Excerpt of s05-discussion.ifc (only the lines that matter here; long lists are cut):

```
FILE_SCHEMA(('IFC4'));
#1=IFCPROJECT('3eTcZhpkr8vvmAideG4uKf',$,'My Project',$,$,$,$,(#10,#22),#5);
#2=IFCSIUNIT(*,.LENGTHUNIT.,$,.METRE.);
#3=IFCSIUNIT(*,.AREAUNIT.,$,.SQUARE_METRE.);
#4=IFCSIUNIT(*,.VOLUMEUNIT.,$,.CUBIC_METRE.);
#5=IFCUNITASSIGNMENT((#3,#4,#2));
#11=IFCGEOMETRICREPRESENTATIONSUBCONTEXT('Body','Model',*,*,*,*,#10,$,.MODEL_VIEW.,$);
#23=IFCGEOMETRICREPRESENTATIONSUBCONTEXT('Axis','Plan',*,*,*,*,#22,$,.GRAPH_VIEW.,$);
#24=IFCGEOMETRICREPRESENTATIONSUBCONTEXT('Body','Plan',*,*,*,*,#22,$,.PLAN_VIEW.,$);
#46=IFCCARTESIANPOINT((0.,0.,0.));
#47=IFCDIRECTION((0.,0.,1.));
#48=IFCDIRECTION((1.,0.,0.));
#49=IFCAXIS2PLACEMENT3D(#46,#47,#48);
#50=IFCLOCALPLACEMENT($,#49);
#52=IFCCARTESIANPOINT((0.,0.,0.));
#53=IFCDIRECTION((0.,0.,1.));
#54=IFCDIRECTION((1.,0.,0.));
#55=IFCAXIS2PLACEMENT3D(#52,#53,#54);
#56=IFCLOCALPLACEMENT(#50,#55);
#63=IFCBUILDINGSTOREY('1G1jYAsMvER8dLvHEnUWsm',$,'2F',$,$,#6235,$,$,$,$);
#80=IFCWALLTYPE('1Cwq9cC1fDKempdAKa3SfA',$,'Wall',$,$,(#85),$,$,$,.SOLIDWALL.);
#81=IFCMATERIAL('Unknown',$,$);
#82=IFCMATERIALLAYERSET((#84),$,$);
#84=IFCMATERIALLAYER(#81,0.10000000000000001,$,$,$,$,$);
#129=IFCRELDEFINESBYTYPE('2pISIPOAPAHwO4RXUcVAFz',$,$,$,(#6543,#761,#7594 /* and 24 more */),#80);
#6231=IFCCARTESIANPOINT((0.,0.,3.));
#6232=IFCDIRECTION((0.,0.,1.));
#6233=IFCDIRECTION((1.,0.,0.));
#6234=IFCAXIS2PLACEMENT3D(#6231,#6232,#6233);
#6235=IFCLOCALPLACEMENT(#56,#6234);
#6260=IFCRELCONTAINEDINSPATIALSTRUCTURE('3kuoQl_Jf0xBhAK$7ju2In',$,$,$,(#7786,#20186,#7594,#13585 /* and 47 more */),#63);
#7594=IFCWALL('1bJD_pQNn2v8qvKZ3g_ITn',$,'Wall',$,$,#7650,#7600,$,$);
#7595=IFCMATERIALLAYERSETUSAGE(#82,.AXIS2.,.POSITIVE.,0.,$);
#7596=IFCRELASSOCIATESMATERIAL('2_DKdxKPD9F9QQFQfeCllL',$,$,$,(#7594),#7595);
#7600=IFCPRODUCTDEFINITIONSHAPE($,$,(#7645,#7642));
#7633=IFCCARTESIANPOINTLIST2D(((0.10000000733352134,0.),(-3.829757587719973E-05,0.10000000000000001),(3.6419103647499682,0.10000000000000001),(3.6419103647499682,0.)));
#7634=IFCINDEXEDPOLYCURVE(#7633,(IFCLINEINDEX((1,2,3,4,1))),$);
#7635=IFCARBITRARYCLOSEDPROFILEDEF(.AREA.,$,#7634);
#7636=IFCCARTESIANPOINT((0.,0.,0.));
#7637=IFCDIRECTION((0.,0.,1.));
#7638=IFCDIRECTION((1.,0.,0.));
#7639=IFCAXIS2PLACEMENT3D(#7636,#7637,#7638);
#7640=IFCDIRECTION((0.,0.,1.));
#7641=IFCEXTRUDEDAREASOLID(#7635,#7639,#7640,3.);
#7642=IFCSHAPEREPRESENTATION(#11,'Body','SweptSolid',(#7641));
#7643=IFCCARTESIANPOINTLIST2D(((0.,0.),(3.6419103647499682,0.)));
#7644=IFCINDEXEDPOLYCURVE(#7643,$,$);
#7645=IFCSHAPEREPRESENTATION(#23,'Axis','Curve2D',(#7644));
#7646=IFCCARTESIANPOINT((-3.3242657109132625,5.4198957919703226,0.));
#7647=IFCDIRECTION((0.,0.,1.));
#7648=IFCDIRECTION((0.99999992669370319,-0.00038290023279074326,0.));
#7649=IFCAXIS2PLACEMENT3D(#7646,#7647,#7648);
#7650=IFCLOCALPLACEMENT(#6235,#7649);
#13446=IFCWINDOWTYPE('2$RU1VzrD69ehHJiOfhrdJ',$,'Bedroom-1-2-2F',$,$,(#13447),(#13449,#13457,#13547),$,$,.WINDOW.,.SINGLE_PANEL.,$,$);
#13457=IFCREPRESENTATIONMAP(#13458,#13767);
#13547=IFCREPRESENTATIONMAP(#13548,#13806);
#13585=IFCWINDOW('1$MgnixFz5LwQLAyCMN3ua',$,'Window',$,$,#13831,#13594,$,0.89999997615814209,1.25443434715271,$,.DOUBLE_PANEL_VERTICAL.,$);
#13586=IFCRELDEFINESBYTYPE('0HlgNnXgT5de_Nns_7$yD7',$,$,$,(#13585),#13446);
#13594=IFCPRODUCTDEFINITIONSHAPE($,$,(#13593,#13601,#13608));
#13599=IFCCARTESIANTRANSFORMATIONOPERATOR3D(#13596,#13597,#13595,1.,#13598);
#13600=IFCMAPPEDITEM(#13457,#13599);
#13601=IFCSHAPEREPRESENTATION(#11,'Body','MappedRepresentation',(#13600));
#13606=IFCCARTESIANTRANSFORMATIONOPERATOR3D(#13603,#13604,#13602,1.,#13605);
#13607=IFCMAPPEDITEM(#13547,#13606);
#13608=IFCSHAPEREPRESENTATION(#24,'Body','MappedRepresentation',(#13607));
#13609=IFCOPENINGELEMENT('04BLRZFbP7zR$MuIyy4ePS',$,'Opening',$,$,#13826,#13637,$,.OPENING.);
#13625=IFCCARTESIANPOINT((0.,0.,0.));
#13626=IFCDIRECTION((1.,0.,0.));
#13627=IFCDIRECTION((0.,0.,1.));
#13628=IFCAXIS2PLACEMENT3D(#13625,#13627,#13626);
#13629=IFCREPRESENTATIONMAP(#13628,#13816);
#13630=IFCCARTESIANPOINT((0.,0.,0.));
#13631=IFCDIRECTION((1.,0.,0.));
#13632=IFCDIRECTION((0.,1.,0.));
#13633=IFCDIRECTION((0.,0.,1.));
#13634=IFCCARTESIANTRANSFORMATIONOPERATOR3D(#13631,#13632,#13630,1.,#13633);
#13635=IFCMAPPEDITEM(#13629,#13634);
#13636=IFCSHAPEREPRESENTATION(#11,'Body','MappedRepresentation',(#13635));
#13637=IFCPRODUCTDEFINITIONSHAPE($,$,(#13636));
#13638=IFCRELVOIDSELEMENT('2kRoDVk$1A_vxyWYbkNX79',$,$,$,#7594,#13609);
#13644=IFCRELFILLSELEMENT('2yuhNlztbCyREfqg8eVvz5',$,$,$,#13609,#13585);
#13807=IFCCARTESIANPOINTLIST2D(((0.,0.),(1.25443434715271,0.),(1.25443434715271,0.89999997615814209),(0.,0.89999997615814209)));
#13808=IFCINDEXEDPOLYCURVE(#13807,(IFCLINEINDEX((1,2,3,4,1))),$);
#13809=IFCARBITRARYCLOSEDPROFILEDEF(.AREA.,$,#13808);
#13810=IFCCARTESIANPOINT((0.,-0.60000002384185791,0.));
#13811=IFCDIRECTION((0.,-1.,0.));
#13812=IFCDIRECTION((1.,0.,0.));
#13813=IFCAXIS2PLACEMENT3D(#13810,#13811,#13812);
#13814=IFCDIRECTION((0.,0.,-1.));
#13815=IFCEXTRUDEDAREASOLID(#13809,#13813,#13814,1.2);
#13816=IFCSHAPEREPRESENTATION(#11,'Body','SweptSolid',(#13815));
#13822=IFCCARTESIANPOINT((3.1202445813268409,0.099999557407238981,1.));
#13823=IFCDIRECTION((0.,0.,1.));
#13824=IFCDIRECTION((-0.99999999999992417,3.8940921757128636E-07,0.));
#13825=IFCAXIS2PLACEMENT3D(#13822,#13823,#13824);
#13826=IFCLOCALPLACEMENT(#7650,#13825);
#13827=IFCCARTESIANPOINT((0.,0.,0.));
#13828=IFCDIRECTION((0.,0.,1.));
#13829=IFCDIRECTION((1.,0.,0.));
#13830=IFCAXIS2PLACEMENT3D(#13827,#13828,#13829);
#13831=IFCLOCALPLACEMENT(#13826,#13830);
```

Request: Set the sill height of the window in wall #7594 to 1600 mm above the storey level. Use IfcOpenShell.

```python
import numpy as np
import ifcopenshell
import ifcopenshell.api.geometry
import ifcopenshell.geom
import ifcopenshell.util.element
import ifcopenshell.util.placement
import ifcopenshell.util.shape
import ifcopenshell.util.unit

model = ifcopenshell.open("s05-discussion.ifc")
unit_scale = ifcopenshell.util.unit.calculate_unit_scale(model)

window = model.by_guid("1$MgnixFz5LwQLAyCMN3ua")
opening = window.FillsVoids[0].RelatingOpeningElement
storey = ifcopenshell.util.element.get_container(window, ifc_class="IfcBuildingStorey")
level = ifcopenshell.util.placement.get_local_placement(storey.ObjectPlacement)[2, 3]

# The opening's origin need not be at the sill, so measure its lowest point.
shape = ifcopenshell.geom.create_shape(ifcopenshell.geom.settings(), opening)
bottom = ifcopenshell.util.shape.get_shape_bottom_elevation(shape, shape.geometry) / unit_scale
dz = level + 1.6 - bottom

shift = np.array([0.0, 0.0, dz])
# The window is placed relative to its opening, so it follows when the opening moves.
matrix = ifcopenshell.util.placement.get_local_placement(opening.ObjectPlacement)
matrix[:3, 3] += shift
ifcopenshell.api.geometry.edit_object_placement(
    model, product=opening, matrix=matrix, is_si=False, should_transform_children=True
)

print(f"moved by {dz * unit_scale:+.3f} m")

model.write("s05-discussion_v2.ifc")
```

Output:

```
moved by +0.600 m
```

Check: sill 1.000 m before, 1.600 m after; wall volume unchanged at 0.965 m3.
